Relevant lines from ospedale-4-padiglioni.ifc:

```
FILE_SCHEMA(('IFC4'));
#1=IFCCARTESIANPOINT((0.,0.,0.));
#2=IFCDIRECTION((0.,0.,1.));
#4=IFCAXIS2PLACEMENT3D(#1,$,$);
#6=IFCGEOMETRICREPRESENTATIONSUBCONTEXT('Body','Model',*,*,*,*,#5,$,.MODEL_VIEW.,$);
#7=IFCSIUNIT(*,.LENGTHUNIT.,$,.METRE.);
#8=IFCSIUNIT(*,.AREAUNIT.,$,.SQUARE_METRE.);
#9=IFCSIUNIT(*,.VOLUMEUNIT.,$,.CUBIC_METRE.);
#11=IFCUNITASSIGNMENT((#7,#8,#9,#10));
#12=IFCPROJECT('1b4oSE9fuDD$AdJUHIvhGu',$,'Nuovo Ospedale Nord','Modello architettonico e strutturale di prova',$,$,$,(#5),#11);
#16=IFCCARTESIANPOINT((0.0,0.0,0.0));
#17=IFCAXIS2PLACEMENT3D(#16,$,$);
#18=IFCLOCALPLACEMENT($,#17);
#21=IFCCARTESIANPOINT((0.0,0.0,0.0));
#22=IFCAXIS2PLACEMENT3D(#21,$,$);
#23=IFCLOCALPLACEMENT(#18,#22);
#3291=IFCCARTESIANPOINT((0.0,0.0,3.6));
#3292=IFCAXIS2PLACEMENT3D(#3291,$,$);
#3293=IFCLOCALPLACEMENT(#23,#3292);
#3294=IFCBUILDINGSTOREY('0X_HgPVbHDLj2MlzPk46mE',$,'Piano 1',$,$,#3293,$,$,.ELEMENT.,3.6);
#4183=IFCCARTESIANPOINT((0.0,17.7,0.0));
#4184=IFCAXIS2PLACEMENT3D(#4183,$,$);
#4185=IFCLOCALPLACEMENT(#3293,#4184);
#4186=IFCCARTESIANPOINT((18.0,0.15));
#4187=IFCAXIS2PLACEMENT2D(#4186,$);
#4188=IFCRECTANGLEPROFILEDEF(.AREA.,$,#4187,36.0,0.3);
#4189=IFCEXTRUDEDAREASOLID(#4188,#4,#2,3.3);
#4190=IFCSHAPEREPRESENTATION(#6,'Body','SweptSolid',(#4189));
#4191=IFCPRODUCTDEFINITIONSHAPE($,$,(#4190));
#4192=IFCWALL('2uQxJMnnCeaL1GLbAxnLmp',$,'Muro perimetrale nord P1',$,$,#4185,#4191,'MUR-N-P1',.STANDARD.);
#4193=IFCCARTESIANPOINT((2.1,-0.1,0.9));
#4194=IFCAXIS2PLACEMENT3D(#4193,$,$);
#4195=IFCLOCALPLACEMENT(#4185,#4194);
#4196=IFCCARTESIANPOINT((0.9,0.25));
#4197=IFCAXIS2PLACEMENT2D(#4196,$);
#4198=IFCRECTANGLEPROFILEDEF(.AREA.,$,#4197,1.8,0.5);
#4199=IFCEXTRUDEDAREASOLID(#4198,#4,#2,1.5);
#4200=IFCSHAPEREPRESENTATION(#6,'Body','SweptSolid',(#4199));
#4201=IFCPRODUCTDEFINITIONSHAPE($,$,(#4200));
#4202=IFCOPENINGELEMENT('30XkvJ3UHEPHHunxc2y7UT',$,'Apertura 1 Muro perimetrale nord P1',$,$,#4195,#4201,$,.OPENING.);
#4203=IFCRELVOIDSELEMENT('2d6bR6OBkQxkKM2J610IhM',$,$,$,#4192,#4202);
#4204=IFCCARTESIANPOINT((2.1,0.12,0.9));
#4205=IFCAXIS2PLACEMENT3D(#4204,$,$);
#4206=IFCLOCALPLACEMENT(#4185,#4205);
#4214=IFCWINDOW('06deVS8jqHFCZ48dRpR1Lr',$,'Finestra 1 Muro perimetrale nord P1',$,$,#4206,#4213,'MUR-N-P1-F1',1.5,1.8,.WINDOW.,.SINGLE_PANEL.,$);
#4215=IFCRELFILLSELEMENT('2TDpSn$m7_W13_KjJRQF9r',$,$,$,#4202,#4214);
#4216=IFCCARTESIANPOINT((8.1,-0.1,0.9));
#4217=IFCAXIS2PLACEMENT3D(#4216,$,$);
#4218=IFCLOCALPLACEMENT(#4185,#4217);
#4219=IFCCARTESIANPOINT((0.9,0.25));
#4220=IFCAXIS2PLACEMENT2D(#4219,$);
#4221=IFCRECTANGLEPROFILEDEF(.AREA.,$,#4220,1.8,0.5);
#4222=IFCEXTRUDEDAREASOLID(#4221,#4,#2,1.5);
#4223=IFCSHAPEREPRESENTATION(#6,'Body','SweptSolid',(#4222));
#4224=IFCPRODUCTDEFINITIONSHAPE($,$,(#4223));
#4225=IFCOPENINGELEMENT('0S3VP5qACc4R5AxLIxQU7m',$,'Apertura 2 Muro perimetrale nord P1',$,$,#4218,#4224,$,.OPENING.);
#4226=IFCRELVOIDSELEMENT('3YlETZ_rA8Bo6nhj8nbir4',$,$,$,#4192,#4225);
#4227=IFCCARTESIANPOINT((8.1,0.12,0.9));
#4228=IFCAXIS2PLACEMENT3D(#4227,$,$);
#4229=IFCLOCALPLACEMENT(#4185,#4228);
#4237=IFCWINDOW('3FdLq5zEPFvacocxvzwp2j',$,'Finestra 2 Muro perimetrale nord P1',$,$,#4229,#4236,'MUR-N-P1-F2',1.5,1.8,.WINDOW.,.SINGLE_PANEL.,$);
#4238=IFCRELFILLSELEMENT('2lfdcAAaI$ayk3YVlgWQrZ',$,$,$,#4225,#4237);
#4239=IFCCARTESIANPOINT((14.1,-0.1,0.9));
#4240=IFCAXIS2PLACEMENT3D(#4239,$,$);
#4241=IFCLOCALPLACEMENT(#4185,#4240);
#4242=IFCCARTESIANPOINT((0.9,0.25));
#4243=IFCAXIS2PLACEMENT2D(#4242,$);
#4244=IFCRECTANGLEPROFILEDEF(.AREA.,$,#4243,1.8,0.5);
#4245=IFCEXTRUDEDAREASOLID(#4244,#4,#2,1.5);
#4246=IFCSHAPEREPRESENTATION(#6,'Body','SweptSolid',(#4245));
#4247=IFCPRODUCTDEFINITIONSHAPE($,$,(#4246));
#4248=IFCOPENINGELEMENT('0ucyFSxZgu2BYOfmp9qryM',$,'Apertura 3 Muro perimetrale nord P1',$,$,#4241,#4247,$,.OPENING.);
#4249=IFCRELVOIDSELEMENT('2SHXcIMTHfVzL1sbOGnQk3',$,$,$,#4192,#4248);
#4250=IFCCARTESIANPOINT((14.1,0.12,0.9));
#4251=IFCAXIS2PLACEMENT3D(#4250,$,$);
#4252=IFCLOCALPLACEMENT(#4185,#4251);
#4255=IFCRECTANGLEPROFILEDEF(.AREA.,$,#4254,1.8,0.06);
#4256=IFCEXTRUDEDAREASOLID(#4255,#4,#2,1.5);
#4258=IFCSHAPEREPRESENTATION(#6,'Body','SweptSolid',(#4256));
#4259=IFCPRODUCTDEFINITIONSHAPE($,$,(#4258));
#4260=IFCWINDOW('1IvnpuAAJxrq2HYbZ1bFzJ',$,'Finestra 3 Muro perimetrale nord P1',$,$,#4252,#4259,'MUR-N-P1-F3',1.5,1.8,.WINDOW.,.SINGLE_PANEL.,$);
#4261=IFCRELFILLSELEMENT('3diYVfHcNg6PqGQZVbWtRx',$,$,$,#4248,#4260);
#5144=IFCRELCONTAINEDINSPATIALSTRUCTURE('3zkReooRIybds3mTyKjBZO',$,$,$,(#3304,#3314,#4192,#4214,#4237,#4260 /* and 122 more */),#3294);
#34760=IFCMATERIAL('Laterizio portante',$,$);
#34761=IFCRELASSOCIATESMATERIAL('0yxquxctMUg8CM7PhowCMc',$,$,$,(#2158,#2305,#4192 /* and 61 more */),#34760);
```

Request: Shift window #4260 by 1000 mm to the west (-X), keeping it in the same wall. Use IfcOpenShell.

```python
import ifcopenshell
import ifcopenshell.api.geometry
import ifcopenshell.util.placement

model = ifcopenshell.open("ospedale-4-padiglioni.ifc")

window = model.by_guid("1IvnpuAAJxrq2HYbZ1bFzJ")
opening = window.FillsVoids[0].RelatingOpeningElement
wall = opening.VoidsElements[0].RelatingBuildingElement

wall_matrix = ifcopenshell.util.placement.get_local_placement(wall.ObjectPlacement)
shift = wall_matrix[:3, 0] * -1.0
before = ifcopenshell.util.placement.get_local_placement(window.ObjectPlacement)[:3, 3].copy()

# The window is not placed relative to its opening, so move both.
for product in (opening, window):
    matrix = ifcopenshell.util.placement.get_local_placement(product.ObjectPlacement)
    matrix[:3, 3] += shift
    ifcopenshell.api.geometry.edit_object_placement(model, product=product, matrix=matrix, is_si=False)

after = ifcopenshell.util.placement.get_local_placement(window.ObjectPlacement)[:3, 3]
print("window moved by", (after - before).round(3) + 0.0)

model.write("ospedale-4-padiglioni_edited.ifc")
```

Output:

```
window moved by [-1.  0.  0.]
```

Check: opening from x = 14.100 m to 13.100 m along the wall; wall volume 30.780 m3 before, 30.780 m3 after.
